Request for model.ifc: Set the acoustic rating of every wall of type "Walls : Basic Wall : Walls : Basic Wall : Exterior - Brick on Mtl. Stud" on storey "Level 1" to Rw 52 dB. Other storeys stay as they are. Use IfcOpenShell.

First a look at what the model holds.

```python
import ifcopenshell
import ifcopenshell.util.element

model = ifcopenshell.open("model.ifc")
print(model.schema)
storey = next(s for s in model.by_type("IfcBuildingStorey") if s.Name == "Level 1")
walls = [e for e in ifcopenshell.util.element.get_decomposition(storey) if e.is_a("IfcWall")]
seen = {}
for e in walls:
    element_type = ifcopenshell.util.element.get_type(e)
    key = (element_type.Name if element_type != e and element_type else None, ifcopenshell.util.element.get_pset(e, "Pset_WallCommon", "AcousticRating"))
    seen[key] = seen.get(key, 0) + 1
for (name, value), count in sorted(seen.items(), key=str):
    print(count, "x", name, "|", value)
```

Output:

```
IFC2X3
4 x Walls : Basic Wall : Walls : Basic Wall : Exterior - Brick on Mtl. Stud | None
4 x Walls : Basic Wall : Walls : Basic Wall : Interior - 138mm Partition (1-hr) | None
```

```python
import ifcopenshell
import ifcopenshell.api.pset
import ifcopenshell.util.element

model = ifcopenshell.open("model.ifc")

storey = next(s for s in model.by_type("IfcBuildingStorey") if s.Name == "Level 1")
walls = [e for e in ifcopenshell.util.element.get_decomposition(storey) if e.is_a("IfcWall")]

count = 0
for e in walls:
    element_type = ifcopenshell.util.element.get_type(e)
    if element_type in (None, e) or element_type.Name != "Walls : Basic Wall : Walls : Basic Wall : Exterior - Brick on Mtl. Stud":
        continue
    # add_pset returns the element's existing set when there is one.
    pset = ifcopenshell.api.pset.add_pset(model, product=e, name="Pset_WallCommon")
    ifcopenshell.api.pset.edit_pset(model, pset=pset, properties={"AcousticRating": "Rw 52 dB"})
    count += 1

print(count, "walls updated")

model.write("model_edited.ifc")
```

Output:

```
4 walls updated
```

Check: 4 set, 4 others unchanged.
